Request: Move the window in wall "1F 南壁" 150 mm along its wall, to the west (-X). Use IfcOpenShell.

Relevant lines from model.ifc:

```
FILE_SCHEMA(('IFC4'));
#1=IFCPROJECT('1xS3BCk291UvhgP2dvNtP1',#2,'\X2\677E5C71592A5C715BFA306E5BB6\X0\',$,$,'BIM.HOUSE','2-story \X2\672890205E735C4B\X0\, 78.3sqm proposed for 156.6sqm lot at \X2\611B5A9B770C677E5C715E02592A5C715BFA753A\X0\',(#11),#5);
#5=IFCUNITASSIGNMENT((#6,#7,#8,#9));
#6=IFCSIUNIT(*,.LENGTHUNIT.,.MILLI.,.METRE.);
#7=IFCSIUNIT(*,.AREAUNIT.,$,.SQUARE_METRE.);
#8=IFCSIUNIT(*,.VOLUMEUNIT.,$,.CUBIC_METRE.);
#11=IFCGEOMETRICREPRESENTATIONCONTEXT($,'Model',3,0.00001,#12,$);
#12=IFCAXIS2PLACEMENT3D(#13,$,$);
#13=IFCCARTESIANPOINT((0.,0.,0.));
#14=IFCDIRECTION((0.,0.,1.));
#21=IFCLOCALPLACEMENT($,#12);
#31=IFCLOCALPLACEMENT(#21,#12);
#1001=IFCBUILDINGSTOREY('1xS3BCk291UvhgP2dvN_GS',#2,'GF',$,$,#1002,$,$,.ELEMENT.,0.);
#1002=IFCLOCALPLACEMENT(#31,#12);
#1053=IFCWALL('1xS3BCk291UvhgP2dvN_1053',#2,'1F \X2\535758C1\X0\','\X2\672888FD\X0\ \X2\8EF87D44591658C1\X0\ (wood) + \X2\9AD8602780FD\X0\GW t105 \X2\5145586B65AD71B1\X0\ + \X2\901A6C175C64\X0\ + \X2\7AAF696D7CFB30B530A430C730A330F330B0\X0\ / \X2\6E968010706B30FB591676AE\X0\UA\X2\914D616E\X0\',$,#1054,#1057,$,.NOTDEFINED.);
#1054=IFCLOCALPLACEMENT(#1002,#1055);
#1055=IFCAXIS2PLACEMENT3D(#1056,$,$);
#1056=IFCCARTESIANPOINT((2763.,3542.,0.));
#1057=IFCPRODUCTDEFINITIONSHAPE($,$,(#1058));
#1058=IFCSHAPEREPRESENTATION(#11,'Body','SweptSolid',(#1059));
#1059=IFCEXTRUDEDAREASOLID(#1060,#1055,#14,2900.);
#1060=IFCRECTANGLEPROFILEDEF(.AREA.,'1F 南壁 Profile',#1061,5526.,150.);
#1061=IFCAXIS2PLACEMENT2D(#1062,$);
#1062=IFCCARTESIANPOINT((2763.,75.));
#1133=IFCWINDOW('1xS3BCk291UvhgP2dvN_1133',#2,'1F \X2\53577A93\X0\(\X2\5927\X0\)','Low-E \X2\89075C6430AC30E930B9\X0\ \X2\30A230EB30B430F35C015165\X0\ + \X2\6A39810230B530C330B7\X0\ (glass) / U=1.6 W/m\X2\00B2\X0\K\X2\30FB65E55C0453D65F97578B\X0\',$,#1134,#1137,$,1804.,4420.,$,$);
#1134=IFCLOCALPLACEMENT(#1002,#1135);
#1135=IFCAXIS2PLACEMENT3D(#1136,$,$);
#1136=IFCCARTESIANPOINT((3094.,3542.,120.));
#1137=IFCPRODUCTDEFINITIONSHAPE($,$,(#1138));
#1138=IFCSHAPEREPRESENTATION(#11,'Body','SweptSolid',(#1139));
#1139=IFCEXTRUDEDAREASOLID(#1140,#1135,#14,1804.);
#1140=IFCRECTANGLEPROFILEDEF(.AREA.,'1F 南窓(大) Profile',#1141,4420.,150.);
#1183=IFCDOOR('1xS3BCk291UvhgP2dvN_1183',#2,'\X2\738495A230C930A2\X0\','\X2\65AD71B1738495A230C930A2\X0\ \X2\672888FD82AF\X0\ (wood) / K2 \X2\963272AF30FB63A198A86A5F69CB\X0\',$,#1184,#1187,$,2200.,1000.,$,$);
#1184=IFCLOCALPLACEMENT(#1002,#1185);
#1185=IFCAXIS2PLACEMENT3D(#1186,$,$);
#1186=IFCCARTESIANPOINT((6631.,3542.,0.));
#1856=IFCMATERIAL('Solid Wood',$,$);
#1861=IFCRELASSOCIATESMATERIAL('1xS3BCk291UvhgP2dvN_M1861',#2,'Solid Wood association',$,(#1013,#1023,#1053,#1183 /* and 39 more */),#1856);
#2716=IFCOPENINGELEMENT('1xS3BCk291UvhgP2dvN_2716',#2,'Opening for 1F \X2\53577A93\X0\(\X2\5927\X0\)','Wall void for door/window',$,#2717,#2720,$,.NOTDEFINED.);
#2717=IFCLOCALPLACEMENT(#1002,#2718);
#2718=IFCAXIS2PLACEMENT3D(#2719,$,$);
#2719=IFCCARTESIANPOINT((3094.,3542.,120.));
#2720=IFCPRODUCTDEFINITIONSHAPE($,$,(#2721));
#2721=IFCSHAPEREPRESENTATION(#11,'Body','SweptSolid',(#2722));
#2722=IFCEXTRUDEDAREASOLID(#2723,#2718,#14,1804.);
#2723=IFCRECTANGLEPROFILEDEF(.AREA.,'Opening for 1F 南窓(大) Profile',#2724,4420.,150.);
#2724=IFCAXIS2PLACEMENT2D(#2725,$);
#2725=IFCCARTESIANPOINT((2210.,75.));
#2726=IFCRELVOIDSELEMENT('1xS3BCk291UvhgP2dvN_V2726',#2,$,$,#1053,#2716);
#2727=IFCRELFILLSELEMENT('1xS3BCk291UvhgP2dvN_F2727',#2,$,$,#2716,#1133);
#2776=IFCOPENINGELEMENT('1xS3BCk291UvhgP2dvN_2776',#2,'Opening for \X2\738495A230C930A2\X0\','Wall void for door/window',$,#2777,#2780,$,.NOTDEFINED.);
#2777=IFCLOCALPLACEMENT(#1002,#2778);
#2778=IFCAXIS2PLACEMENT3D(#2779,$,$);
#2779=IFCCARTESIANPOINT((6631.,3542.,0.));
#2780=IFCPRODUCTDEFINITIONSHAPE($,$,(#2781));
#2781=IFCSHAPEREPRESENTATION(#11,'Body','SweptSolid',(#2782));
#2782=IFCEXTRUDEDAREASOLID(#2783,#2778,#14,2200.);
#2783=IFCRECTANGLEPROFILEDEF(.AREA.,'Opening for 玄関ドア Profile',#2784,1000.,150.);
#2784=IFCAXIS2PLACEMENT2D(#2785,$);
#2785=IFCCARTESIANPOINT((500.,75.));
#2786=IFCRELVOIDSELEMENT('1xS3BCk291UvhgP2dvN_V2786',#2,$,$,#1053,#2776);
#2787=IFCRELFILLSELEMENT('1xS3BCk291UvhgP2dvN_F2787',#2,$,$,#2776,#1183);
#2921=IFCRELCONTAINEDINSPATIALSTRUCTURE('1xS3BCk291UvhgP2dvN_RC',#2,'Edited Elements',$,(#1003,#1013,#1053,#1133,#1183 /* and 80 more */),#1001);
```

```python
import ifcopenshell
import ifcopenshell.api.geometry
import ifcopenshell.util.placement
import ifcopenshell.util.unit

model = ifcopenshell.open("model.ifc")
unit_scale = ifcopenshell.util.unit.calculate_unit_scale(model)

window = model.by_guid("1xS3BCk291UvhgP2dvN_1133")
opening = window.FillsVoids[0].RelatingOpeningElement
wall = opening.VoidsElements[0].RelatingBuildingElement

wall_matrix = ifcopenshell.util.placement.get_local_placement(wall.ObjectPlacement)
shift = wall_matrix[:3, 0] * -0.15 / unit_scale
before = ifcopenshell.util.placement.get_local_placement(window.ObjectPlacement)[:3, 3].copy()

# The window is not placed relative to its opening, so move both.
for product in (opening, window):
    matrix = ifcopenshell.util.placement.get_local_placement(product.ObjectPlacement)
    matrix[:3, 3] += shift
    ifcopenshell.api.geometry.edit_object_placement(model, product=product, matrix=matrix, is_si=False)

after = ifcopenshell.util.placement.get_local_placement(window.ObjectPlacement)[:3, 3]
print("window moved by", (after - before).round(3) + 0.0)

model.write("model_v2.ifc")
```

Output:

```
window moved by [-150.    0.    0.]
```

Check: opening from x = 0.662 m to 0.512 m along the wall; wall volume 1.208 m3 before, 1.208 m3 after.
